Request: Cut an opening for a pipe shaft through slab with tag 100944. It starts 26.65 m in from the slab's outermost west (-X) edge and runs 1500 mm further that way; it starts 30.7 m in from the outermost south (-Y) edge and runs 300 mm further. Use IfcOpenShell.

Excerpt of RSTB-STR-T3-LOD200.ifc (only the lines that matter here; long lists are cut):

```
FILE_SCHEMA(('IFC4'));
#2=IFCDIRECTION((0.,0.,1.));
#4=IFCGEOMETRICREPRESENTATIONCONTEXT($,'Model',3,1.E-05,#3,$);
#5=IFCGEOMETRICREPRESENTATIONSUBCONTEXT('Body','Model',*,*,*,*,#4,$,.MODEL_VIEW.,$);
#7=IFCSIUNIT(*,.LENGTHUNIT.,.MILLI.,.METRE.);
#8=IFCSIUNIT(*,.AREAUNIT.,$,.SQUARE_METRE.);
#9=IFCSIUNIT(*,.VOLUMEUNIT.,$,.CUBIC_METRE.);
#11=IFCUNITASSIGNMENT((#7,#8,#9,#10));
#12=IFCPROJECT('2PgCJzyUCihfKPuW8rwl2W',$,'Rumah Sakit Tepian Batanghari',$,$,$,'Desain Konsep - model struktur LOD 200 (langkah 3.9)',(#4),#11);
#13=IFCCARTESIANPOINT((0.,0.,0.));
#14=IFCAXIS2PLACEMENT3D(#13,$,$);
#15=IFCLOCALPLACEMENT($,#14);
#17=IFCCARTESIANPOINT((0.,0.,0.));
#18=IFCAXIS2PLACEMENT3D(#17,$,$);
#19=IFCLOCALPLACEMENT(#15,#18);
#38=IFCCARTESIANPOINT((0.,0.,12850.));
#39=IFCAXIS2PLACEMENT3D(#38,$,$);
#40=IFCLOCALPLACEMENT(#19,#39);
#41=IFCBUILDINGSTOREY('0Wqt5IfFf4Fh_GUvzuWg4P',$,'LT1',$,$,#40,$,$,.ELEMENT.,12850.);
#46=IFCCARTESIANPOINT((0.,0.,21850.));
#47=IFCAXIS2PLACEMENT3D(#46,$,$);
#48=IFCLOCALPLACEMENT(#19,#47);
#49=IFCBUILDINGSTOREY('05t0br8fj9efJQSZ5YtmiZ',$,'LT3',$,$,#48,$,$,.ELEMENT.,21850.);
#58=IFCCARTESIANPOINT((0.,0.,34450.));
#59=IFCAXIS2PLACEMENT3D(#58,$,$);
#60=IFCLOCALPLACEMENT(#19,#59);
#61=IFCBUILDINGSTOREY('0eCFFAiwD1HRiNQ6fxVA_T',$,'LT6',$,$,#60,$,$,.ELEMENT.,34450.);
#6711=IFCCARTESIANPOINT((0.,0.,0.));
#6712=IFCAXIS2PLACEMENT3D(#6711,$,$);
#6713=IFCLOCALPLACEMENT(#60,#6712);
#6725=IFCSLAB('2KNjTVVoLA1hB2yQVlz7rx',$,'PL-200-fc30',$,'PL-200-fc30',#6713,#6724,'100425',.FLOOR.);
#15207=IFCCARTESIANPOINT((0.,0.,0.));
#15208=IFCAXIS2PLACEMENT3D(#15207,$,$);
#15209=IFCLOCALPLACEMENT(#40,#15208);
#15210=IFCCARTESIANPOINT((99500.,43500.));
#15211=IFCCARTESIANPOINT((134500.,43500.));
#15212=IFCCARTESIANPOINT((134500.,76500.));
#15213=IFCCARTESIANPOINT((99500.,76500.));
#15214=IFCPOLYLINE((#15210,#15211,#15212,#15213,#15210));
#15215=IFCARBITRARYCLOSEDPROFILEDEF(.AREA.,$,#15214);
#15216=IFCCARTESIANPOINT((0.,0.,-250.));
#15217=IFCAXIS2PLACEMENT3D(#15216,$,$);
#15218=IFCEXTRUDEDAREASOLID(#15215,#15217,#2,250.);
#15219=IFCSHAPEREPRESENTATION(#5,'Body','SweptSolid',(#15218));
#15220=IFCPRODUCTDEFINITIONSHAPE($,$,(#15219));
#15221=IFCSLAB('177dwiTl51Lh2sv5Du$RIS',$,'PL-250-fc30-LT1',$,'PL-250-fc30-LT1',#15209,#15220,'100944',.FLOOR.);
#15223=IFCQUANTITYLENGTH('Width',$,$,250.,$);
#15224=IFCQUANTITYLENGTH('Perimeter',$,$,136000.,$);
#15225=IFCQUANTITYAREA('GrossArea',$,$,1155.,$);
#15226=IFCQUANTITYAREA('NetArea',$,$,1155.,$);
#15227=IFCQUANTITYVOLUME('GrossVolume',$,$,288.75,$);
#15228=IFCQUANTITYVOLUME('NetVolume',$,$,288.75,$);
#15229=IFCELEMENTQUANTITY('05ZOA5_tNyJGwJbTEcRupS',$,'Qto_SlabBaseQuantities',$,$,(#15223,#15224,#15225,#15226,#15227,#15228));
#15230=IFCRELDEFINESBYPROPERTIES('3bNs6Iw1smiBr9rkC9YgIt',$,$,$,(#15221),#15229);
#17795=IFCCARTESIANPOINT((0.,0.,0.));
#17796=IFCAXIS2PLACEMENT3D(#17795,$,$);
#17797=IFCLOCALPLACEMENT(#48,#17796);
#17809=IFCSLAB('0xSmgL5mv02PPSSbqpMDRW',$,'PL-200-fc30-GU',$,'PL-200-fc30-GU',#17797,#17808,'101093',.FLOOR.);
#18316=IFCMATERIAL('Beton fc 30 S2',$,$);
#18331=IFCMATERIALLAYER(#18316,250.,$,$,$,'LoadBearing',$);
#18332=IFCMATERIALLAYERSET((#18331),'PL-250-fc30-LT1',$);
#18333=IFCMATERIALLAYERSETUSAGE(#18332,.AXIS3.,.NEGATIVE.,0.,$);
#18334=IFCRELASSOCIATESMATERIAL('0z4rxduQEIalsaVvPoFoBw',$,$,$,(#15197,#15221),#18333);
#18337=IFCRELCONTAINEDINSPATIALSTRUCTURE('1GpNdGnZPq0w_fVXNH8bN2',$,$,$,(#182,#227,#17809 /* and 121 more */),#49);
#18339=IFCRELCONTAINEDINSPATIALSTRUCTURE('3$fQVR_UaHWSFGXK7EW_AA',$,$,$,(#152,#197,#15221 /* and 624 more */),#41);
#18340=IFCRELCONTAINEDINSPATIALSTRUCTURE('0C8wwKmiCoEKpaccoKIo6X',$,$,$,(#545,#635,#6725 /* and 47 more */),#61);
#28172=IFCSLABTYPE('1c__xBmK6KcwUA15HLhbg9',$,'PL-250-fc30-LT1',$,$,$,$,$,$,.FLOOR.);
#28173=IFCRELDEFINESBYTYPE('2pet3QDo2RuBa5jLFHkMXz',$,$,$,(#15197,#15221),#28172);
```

```python
import numpy as np
import ifcopenshell
import ifcopenshell.api.feature
import ifcopenshell.api.geometry
import ifcopenshell.api.pset
import ifcopenshell.api.root
import ifcopenshell.geom
import ifcopenshell.util.element
import ifcopenshell.util.placement
import ifcopenshell.util.representation
import ifcopenshell.util.shape
import ifcopenshell.util.unit

model = ifcopenshell.open("RSTB-STR-T3-LOD200.ifc")
unit_scale = ifcopenshell.util.unit.calculate_unit_scale(model)
area_scale = ifcopenshell.util.unit.calculate_unit_scale(model, "AREAUNIT")
volume_scale = ifcopenshell.util.unit.calculate_unit_scale(model, "VOLUMEUNIT")
settings = ifcopenshell.geom.settings()


def volume(element):
    """Net volume in cubic metres, openings subtracted."""
    shape = ifcopenshell.geom.create_shape(settings, element)
    return ifcopenshell.util.shape.get_volume(shape.geometry)


slab = model.by_guid("177dwiTl51Lh2sv5Du$RIS")
before = volume(slab)

# Extent in the slab's own axes, in metres. The edges named are its -X and -Y sides.
slab_shape = ifcopenshell.geom.create_shape(settings, slab)
vertices = ifcopenshell.util.shape.get_vertices(slab_shape.geometry)
x_min, y_min, bottom = vertices.min(axis=0)
top = vertices[:, 2].max()

opening = ifcopenshell.api.root.create_entity(model, ifc_class="IfcOpeningElement", name="Pipe shaft opening", predefined_type="OPENING")
context = ifcopenshell.util.representation.get_context(model, "Model", "Body", "MODEL_VIEW")
width, depth = 1.5, 0.3
outline = [(0.0, 0.0), (width, 0.0), (width, depth), (0.0, depth), (0.0, 0.0)]
# Overshoot both faces by 50 mm so the cut is clean.
shape = ifcopenshell.api.geometry.add_slab_representation(
    model, context=context, depth=top - bottom + 0.1, polyline=outline
)
ifcopenshell.api.geometry.assign_representation(model, product=opening, representation=shape)

matrix = ifcopenshell.util.placement.get_local_placement(slab.ObjectPlacement)
matrix[:, 3] = matrix @ np.append(np.array([x_min + 26.65, y_min + 30.7, bottom - 0.05]) / unit_scale, 1.0)
ifcopenshell.api.geometry.edit_object_placement(model, product=opening, matrix=matrix, is_si=False)
ifcopenshell.api.feature.add_feature(model, feature=opening, element=slab)

after = volume(slab)

# Update the slab's stored quantities.
qto = model.by_id(ifcopenshell.util.element.get_pset(slab, "Qto_SlabBaseQuantities", should_inherit=False)["id"])
ifcopenshell.api.pset.edit_qto(model, qto=qto, properties={
    "NetArea": after / (top - bottom) / area_scale,
    "NetVolume": after / volume_scale,
})

print(f"slab volume {before:.3f} -> {after:.3f} m3")

model.write("RSTB-STR-T3-LOD200_updated.ifc")
```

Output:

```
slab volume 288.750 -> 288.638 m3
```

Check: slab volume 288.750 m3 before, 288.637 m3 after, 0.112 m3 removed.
